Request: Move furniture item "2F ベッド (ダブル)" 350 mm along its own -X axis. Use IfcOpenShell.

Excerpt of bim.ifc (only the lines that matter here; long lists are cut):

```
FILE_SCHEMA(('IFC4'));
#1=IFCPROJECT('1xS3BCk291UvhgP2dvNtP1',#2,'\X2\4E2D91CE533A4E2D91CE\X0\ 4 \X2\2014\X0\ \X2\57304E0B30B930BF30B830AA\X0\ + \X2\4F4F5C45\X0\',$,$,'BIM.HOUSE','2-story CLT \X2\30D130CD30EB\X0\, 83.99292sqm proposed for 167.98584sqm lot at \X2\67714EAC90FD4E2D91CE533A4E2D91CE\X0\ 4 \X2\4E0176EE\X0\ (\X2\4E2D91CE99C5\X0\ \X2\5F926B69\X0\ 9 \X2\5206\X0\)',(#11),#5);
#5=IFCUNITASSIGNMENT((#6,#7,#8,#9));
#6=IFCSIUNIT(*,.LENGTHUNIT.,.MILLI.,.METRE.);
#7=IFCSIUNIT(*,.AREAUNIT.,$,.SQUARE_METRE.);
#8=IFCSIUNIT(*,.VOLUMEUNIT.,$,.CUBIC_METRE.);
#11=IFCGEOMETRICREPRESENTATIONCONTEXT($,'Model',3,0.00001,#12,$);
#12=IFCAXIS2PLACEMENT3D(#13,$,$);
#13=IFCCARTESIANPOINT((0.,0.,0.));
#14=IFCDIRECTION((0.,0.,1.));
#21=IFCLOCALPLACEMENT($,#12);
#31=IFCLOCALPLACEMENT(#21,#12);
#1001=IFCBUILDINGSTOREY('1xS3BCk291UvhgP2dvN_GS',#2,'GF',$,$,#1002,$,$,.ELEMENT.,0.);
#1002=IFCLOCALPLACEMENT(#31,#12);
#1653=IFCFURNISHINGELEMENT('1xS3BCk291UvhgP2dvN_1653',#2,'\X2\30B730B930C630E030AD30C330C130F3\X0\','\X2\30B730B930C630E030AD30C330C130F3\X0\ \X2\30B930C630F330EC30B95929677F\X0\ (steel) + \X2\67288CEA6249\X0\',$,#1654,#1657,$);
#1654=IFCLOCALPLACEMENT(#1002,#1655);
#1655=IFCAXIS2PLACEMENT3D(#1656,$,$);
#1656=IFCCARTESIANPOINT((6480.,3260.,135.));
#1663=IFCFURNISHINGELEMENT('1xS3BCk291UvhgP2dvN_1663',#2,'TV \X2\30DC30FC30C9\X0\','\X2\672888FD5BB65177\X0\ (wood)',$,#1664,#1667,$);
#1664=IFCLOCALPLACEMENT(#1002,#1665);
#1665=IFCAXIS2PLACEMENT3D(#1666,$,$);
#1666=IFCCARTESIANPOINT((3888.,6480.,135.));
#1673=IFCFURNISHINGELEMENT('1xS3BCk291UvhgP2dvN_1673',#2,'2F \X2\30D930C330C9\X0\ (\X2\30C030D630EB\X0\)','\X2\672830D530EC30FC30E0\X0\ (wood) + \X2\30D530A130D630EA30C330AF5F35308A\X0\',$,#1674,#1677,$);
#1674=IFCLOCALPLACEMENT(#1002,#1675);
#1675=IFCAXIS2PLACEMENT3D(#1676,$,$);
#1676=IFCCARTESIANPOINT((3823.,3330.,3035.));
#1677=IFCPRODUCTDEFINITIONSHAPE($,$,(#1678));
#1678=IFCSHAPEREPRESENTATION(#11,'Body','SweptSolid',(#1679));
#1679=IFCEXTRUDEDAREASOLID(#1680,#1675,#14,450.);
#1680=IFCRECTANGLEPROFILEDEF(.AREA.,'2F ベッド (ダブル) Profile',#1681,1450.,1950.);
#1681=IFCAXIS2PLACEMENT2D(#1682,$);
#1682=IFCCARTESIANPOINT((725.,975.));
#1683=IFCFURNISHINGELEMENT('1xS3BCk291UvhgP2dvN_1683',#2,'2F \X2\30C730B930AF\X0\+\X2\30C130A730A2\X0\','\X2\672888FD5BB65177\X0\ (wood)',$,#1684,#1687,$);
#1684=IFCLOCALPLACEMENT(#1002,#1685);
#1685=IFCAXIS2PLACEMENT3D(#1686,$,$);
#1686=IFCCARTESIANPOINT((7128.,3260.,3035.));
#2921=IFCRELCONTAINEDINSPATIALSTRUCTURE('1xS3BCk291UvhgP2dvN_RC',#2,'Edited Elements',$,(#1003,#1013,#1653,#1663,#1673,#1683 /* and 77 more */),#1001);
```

```python
import ifcopenshell
import ifcopenshell.api.geometry
import ifcopenshell.util.placement
import ifcopenshell.util.unit

model = ifcopenshell.open("bim.ifc")
unit_scale = ifcopenshell.util.unit.calculate_unit_scale(model)

item = model.by_guid("1xS3BCk291UvhgP2dvN_1673")
matrix = ifcopenshell.util.placement.get_local_placement(item.ObjectPlacement)
matrix[:3, 3] -= matrix[:3, 0] * 0.35 / unit_scale
ifcopenshell.api.geometry.edit_object_placement(model, product=item, matrix=matrix, is_si=False)

print(ifcopenshell.util.placement.get_local_placement(item.ObjectPlacement).round(3) + 0.0)

model.write("bim_edited.ifc")
```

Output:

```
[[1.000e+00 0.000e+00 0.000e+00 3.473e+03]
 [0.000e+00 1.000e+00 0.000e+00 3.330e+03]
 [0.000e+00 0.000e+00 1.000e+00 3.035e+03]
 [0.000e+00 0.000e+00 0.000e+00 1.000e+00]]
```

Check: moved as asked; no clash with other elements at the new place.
